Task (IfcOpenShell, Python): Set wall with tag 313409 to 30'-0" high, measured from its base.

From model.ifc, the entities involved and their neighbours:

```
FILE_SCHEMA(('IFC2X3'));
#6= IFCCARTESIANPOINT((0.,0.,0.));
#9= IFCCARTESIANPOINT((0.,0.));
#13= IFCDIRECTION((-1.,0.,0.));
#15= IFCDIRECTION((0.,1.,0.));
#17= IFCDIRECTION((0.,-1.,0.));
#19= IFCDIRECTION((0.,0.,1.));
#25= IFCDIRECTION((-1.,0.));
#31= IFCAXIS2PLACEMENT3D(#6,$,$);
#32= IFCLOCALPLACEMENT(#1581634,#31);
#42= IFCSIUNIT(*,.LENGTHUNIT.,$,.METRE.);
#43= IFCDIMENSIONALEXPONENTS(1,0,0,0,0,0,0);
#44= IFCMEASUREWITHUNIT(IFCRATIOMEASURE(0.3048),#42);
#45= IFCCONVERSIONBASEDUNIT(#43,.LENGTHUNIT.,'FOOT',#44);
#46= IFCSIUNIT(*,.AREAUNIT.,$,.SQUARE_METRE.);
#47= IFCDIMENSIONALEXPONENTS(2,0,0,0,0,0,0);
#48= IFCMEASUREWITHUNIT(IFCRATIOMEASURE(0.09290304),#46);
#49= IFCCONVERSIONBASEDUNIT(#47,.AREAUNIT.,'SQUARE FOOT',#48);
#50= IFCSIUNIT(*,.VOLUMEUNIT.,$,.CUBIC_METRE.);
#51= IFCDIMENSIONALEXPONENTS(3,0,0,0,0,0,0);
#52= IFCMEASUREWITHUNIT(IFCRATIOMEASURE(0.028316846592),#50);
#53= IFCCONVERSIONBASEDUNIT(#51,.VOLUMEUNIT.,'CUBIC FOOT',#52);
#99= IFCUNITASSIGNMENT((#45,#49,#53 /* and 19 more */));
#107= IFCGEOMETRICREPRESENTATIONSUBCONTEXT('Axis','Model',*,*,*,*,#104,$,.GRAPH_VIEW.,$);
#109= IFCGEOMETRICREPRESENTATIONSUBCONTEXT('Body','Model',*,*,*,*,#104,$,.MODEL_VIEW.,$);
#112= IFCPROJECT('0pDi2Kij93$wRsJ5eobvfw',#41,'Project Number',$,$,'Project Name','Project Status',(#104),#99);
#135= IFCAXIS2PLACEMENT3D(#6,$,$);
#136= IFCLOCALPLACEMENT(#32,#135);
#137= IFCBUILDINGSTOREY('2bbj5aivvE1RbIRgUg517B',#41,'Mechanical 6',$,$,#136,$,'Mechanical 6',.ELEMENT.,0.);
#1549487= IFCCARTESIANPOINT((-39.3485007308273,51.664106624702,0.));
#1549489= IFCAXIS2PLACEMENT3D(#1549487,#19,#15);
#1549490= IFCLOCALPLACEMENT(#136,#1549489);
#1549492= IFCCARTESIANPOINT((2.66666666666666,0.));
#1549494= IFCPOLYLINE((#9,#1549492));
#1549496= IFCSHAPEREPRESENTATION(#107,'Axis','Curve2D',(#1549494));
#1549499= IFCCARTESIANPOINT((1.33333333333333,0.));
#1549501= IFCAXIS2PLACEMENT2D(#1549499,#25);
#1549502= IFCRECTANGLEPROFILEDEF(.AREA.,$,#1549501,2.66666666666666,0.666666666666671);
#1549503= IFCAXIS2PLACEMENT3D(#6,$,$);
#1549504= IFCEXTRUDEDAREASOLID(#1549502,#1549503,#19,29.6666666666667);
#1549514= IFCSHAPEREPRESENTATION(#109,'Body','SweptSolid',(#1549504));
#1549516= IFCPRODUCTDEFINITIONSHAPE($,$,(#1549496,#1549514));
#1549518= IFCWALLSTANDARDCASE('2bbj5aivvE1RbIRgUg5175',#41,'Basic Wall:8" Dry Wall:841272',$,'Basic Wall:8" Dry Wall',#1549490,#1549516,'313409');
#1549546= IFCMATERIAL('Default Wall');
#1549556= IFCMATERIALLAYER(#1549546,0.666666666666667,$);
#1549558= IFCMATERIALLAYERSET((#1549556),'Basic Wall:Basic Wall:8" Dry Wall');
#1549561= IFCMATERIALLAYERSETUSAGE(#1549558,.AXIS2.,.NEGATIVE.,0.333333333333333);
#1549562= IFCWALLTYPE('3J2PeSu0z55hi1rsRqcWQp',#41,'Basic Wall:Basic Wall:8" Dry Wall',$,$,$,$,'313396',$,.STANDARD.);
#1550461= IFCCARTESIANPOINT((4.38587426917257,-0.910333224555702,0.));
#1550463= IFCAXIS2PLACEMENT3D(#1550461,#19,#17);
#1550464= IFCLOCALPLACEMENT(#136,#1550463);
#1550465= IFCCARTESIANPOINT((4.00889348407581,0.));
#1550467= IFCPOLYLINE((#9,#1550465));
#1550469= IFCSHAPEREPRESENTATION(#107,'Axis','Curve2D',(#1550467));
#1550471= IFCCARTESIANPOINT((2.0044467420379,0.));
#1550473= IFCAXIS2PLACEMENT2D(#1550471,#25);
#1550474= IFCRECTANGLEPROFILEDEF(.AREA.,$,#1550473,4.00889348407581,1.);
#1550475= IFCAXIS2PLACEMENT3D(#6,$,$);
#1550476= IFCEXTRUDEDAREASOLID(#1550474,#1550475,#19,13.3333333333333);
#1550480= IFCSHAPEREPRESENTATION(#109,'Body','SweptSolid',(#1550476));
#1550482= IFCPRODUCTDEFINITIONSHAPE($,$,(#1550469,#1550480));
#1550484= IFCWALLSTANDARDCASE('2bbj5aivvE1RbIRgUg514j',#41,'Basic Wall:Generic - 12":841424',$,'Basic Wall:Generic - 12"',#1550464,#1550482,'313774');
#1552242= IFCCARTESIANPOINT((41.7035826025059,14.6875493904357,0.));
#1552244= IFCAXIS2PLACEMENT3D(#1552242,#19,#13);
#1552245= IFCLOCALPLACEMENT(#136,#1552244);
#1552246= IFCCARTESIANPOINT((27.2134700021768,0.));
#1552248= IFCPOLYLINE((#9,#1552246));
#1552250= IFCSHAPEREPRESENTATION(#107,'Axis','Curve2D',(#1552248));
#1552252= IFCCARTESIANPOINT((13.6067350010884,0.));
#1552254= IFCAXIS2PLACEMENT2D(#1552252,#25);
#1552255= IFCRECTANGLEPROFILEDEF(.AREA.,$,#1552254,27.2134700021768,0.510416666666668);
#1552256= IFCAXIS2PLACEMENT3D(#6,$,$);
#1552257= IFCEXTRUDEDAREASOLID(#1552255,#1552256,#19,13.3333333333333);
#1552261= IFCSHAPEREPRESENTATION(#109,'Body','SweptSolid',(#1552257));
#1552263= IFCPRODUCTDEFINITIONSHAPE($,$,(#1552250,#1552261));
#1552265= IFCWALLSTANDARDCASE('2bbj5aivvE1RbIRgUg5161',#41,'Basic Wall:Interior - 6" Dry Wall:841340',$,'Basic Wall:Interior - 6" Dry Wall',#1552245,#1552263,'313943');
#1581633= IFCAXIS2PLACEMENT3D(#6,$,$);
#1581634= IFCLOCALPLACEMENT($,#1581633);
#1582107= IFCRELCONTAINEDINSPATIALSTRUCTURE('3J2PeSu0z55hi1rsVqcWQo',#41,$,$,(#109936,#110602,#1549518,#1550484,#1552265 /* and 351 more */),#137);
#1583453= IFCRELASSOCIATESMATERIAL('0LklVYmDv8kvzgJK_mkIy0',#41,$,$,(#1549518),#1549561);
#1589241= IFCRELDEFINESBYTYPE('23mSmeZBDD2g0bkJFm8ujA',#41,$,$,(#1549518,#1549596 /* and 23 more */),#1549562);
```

```python
import ifcopenshell
import ifcopenshell.geom
import ifcopenshell.util.representation
import ifcopenshell.util.shape
import ifcopenshell.util.unit

model = ifcopenshell.open("model.ifc")
unit_scale = ifcopenshell.util.unit.calculate_unit_scale(model)
settings = ifcopenshell.geom.settings()


def volume(element):
    """Net volume in cubic metres, openings subtracted."""
    shape = ifcopenshell.geom.create_shape(settings, element)
    return ifcopenshell.util.shape.get_volume(shape.geometry)


wall = model.by_guid("2bbj5aivvE1RbIRgUg5175")
before = volume(wall)

body = ifcopenshell.util.representation.get_representation(wall, "Model", "Body")
solid = body.Items[0]
old_height = solid.Depth
solid.Depth = 360 * 0.0254 / unit_scale
after = volume(wall)

print(f"height {old_height:g} -> {solid.Depth:g}, volume {before:.3f} -> {after:.3f} m3")

model.write("model-out.ifc")
```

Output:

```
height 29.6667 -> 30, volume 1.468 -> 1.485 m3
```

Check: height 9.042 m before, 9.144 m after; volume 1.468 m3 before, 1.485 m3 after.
